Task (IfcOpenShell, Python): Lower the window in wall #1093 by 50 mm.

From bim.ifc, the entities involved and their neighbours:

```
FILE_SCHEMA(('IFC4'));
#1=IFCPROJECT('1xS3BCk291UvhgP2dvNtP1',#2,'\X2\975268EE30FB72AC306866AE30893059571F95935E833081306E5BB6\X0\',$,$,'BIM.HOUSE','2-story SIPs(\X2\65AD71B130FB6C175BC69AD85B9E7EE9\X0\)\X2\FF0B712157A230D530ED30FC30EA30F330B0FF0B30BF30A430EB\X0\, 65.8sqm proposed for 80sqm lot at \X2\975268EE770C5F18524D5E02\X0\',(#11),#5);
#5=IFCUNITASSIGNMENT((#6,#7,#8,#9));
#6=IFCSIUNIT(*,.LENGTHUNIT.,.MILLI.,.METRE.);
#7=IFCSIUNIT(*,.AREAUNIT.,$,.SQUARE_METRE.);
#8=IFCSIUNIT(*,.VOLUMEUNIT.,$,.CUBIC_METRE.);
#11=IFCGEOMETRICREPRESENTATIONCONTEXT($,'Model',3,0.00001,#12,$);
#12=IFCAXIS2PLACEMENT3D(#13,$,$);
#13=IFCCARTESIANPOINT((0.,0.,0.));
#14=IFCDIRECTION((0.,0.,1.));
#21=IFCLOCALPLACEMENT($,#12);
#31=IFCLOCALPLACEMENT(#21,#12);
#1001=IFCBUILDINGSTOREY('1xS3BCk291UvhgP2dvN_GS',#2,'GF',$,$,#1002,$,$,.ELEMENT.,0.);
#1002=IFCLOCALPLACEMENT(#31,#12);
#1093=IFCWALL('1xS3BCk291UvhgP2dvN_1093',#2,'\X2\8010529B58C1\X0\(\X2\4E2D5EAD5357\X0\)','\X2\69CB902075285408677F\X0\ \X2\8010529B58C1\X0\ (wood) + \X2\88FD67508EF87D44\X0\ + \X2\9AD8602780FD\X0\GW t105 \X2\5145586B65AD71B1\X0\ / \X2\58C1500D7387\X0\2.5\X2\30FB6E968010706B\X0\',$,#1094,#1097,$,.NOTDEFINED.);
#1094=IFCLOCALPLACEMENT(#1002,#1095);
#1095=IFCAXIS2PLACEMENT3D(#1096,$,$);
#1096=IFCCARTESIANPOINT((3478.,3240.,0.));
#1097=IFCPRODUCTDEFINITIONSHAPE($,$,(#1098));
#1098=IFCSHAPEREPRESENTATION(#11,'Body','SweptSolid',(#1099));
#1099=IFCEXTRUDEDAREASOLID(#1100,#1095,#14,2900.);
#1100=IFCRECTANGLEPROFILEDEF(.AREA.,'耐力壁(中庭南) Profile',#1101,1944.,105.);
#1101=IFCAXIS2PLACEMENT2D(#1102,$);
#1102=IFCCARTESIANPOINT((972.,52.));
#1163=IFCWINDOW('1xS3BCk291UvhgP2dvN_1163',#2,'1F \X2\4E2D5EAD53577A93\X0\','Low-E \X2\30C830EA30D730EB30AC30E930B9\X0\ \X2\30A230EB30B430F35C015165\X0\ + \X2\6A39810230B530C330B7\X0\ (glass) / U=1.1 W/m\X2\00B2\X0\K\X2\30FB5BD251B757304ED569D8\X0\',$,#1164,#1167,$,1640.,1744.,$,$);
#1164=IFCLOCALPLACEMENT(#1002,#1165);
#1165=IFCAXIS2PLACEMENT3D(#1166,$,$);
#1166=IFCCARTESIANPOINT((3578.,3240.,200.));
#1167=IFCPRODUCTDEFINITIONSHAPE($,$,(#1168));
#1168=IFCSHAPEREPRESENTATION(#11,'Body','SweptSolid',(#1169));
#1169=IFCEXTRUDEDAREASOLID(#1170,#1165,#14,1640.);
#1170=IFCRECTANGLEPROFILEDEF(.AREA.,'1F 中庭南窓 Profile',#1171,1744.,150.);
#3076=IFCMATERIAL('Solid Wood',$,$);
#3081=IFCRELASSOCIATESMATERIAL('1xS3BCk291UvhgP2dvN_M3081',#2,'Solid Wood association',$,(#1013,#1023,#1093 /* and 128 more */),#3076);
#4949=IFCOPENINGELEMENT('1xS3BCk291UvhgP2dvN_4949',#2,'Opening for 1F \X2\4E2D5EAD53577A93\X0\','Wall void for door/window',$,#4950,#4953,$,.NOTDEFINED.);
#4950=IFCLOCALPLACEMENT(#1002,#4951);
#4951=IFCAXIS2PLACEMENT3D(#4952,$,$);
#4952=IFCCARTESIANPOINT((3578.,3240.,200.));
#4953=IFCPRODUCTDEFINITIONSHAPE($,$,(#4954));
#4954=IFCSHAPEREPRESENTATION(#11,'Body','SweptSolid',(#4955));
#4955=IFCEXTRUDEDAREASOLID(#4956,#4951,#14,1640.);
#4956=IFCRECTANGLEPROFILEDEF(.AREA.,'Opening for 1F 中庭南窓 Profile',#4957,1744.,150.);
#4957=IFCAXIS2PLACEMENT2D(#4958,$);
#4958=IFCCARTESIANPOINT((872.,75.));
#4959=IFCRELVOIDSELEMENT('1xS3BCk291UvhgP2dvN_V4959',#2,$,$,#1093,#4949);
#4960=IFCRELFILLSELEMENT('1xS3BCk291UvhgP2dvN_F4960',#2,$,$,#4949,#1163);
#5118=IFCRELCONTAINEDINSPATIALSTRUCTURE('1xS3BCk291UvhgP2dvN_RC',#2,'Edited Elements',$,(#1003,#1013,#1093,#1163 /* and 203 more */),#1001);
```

```python
import numpy as np
import ifcopenshell
import ifcopenshell.api.geometry
import ifcopenshell.util.placement
import ifcopenshell.util.unit

model = ifcopenshell.open("bim.ifc")
unit_scale = ifcopenshell.util.unit.calculate_unit_scale(model)

window = model.by_id(1163)
opening = window.FillsVoids[0].RelatingOpeningElement
dz = -50.0

shift = np.array([0.0, 0.0, dz])
# The window is not placed relative to its opening, so move both.
for product in (opening, window):
    matrix = ifcopenshell.util.placement.get_local_placement(product.ObjectPlacement)
    matrix[:3, 3] += shift
    ifcopenshell.api.geometry.edit_object_placement(model, product=product, matrix=matrix, is_si=False)

print(f"moved by {dz * unit_scale:+.3f} m")

model.write("bim_edited.ifc")
```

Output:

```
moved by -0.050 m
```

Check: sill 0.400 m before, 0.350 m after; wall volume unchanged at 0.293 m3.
